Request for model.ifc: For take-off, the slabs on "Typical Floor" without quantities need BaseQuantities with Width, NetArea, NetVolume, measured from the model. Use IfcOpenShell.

First a look at what the model holds.

```python
import ifcopenshell
import ifcopenshell.util.element
import ifcopenshell.util.unit

model = ifcopenshell.open("model.ifc")
print(model.schema)
for unit_type in ("LENGTHUNIT", "AREAUNIT", "VOLUMEUNIT"):
    print(unit_type, ifcopenshell.util.unit.calculate_unit_scale(model, unit_type))
storey = next(s for s in model.by_type("IfcBuildingStorey") if s.Name == "Typical Floor")
slabs = [e for e in ifcopenshell.util.element.get_decomposition(storey) if e.is_a("IfcSlab")]
for e in sorted(slabs, key=lambda e: e.id()):
    print(e.id(), e.is_a(), e.Name, list(ifcopenshell.util.element.get_psets(e, qtos_only=True)), sep=" | ")
```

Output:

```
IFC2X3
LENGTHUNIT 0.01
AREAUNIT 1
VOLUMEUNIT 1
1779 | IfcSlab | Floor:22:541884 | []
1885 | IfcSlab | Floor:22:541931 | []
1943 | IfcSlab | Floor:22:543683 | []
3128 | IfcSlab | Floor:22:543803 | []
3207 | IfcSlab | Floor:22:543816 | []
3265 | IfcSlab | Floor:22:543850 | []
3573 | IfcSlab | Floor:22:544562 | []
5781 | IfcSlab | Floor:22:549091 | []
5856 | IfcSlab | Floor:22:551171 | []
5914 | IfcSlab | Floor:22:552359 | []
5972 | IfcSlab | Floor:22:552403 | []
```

```python
import ifcopenshell
import ifcopenshell.api.pset
import ifcopenshell.geom
import ifcopenshell.util.element
import ifcopenshell.util.shape
import ifcopenshell.util.unit

model = ifcopenshell.open("model.ifc")
unit_scale = ifcopenshell.util.unit.calculate_unit_scale(model)
area_scale = ifcopenshell.util.unit.calculate_unit_scale(model, "AREAUNIT")
volume_scale = ifcopenshell.util.unit.calculate_unit_scale(model, "VOLUMEUNIT")
settings = ifcopenshell.geom.settings()

storey = next(s for s in model.by_type("IfcBuildingStorey") if s.Name == "Typical Floor")
slabs = [e for e in ifcopenshell.util.element.get_decomposition(storey) if e.is_a("IfcSlab")]

for e in sorted(slabs, key=lambda e: e.id()):
    if ifcopenshell.util.element.get_psets(e, qtos_only=True, should_inherit=False):
        continue
    # Geometry comes back in metres, in the element's own axes.
    shape = ifcopenshell.geom.create_shape(settings, e)
    values = {
        "Width": ifcopenshell.util.shape.get_z(shape.geometry) / unit_scale,
        "NetArea": ifcopenshell.util.shape.get_footprint_area(shape.geometry) / area_scale,
        "NetVolume": ifcopenshell.util.shape.get_volume(shape.geometry) / volume_scale,
    }
    qto = ifcopenshell.api.pset.add_qto(model, product=e, name="BaseQuantities")
    ifcopenshell.api.pset.edit_qto(model, qto=qto, properties=values)
    print(e.id(), {k: round(v, 3) for k, v in values.items()})

model.write("model_v2.ifc")
```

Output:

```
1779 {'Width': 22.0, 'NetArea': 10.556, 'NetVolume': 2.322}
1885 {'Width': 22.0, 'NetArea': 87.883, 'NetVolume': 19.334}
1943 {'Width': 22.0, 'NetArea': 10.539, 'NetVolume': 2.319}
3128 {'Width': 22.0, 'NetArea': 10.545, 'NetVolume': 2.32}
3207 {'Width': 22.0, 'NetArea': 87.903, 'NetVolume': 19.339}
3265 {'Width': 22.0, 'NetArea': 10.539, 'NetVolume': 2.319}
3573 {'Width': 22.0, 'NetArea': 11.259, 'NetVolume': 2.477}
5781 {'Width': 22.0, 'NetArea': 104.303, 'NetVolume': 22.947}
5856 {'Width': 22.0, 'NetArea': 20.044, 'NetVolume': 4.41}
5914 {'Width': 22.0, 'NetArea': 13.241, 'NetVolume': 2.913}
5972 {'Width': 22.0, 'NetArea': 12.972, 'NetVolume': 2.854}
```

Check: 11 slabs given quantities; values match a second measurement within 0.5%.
